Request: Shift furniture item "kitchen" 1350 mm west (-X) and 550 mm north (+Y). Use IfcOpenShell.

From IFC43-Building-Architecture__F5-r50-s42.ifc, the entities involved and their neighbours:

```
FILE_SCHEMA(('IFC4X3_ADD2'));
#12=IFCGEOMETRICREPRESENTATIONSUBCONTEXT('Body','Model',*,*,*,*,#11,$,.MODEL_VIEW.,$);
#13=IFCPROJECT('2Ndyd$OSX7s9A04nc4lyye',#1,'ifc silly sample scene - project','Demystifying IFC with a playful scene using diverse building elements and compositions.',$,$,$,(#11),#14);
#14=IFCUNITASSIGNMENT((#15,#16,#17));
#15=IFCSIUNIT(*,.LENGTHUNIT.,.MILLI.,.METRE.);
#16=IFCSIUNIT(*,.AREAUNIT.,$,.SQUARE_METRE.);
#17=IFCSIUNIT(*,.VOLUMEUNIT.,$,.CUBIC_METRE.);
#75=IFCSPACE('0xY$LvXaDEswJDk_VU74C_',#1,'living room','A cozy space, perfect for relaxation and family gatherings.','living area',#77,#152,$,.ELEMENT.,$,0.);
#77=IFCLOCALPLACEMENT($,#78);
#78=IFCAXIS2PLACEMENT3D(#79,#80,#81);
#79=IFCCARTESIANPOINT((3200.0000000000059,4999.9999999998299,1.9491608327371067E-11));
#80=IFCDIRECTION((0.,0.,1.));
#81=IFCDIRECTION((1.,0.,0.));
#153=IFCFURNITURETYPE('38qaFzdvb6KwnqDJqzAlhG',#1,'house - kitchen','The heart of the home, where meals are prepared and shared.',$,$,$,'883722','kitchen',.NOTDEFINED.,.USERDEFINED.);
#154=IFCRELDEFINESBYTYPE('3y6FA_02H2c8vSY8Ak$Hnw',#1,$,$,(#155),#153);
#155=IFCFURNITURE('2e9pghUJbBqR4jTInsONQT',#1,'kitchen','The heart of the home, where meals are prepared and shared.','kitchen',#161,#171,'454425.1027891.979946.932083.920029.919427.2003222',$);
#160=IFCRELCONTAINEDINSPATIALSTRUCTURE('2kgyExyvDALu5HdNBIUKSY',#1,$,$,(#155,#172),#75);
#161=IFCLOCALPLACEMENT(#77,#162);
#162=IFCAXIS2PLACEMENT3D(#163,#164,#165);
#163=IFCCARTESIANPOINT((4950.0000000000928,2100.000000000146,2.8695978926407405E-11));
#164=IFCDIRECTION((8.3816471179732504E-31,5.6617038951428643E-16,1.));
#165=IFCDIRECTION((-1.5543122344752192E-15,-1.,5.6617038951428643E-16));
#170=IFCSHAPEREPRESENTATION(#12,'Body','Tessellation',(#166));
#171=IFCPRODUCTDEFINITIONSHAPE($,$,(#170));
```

```python
import ifcopenshell
import ifcopenshell.api.geometry
import ifcopenshell.util.placement
import ifcopenshell.util.unit

model = ifcopenshell.open("IFC43-Building-Architecture__F5-r50-s42.ifc")
unit_scale = ifcopenshell.util.unit.calculate_unit_scale(model)

item = model.by_id(155)
matrix = ifcopenshell.util.placement.get_local_placement(item.ObjectPlacement)
matrix[0, 3] -= 1.35 / unit_scale
matrix[1, 3] += 0.55 / unit_scale
ifcopenshell.api.geometry.edit_object_placement(model, product=item, matrix=matrix, is_si=False)

print(ifcopenshell.util.placement.get_local_placement(item.ObjectPlacement).round(3) + 0.0)

model.write("IFC43-Building-Architecture__F5-r50-s42-out.ifc")
```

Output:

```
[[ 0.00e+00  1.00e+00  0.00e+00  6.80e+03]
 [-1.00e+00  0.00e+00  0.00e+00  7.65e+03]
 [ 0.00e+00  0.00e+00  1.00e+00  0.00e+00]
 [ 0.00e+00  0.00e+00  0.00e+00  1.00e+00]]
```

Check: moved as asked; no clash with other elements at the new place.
